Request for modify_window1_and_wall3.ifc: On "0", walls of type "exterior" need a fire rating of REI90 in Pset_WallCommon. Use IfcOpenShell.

First a look at what the model holds.

```python
import ifcopenshell
import ifcopenshell.util.element

model = ifcopenshell.open("modify_window1_and_wall3.ifc")
print(model.schema)
storey = next(s for s in model.by_type("IfcBuildingStorey") if s.Name == "0")
walls = [e for e in ifcopenshell.util.element.get_decomposition(storey) if e.is_a("IfcWall")]
seen = {}
for e in walls:
    element_type = ifcopenshell.util.element.get_type(e)
    key = (element_type.Name if element_type != e and element_type else None, ifcopenshell.util.element.get_pset(e, "Pset_WallCommon", "FireRating"))
    seen[key] = seen.get(key, 0) + 1
for (name, value), count in sorted(seen.items(), key=str):
    print(count, "x", name, "|", value)
```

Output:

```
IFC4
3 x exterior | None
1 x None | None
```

```python
import ifcopenshell
import ifcopenshell.api.pset
import ifcopenshell.util.element

model = ifcopenshell.open("modify_window1_and_wall3.ifc")

storey = next(s for s in model.by_type("IfcBuildingStorey") if s.Name == "0")
walls = [e for e in ifcopenshell.util.element.get_decomposition(storey) if e.is_a("IfcWall")]

count = 0
for e in walls:
    element_type = ifcopenshell.util.element.get_type(e)
    if element_type in (None, e) or element_type.Name != "exterior":
        continue
    # add_pset returns the element's existing set when there is one.
    pset = ifcopenshell.api.pset.add_pset(model, product=e, name="Pset_WallCommon")
    ifcopenshell.api.pset.edit_pset(model, pset=pset, properties={"FireRating": "REI90"})
    count += 1

print(count, "walls updated")

model.write("modify_window1_and_wall3_updated.ifc")
```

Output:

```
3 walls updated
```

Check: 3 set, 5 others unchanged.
